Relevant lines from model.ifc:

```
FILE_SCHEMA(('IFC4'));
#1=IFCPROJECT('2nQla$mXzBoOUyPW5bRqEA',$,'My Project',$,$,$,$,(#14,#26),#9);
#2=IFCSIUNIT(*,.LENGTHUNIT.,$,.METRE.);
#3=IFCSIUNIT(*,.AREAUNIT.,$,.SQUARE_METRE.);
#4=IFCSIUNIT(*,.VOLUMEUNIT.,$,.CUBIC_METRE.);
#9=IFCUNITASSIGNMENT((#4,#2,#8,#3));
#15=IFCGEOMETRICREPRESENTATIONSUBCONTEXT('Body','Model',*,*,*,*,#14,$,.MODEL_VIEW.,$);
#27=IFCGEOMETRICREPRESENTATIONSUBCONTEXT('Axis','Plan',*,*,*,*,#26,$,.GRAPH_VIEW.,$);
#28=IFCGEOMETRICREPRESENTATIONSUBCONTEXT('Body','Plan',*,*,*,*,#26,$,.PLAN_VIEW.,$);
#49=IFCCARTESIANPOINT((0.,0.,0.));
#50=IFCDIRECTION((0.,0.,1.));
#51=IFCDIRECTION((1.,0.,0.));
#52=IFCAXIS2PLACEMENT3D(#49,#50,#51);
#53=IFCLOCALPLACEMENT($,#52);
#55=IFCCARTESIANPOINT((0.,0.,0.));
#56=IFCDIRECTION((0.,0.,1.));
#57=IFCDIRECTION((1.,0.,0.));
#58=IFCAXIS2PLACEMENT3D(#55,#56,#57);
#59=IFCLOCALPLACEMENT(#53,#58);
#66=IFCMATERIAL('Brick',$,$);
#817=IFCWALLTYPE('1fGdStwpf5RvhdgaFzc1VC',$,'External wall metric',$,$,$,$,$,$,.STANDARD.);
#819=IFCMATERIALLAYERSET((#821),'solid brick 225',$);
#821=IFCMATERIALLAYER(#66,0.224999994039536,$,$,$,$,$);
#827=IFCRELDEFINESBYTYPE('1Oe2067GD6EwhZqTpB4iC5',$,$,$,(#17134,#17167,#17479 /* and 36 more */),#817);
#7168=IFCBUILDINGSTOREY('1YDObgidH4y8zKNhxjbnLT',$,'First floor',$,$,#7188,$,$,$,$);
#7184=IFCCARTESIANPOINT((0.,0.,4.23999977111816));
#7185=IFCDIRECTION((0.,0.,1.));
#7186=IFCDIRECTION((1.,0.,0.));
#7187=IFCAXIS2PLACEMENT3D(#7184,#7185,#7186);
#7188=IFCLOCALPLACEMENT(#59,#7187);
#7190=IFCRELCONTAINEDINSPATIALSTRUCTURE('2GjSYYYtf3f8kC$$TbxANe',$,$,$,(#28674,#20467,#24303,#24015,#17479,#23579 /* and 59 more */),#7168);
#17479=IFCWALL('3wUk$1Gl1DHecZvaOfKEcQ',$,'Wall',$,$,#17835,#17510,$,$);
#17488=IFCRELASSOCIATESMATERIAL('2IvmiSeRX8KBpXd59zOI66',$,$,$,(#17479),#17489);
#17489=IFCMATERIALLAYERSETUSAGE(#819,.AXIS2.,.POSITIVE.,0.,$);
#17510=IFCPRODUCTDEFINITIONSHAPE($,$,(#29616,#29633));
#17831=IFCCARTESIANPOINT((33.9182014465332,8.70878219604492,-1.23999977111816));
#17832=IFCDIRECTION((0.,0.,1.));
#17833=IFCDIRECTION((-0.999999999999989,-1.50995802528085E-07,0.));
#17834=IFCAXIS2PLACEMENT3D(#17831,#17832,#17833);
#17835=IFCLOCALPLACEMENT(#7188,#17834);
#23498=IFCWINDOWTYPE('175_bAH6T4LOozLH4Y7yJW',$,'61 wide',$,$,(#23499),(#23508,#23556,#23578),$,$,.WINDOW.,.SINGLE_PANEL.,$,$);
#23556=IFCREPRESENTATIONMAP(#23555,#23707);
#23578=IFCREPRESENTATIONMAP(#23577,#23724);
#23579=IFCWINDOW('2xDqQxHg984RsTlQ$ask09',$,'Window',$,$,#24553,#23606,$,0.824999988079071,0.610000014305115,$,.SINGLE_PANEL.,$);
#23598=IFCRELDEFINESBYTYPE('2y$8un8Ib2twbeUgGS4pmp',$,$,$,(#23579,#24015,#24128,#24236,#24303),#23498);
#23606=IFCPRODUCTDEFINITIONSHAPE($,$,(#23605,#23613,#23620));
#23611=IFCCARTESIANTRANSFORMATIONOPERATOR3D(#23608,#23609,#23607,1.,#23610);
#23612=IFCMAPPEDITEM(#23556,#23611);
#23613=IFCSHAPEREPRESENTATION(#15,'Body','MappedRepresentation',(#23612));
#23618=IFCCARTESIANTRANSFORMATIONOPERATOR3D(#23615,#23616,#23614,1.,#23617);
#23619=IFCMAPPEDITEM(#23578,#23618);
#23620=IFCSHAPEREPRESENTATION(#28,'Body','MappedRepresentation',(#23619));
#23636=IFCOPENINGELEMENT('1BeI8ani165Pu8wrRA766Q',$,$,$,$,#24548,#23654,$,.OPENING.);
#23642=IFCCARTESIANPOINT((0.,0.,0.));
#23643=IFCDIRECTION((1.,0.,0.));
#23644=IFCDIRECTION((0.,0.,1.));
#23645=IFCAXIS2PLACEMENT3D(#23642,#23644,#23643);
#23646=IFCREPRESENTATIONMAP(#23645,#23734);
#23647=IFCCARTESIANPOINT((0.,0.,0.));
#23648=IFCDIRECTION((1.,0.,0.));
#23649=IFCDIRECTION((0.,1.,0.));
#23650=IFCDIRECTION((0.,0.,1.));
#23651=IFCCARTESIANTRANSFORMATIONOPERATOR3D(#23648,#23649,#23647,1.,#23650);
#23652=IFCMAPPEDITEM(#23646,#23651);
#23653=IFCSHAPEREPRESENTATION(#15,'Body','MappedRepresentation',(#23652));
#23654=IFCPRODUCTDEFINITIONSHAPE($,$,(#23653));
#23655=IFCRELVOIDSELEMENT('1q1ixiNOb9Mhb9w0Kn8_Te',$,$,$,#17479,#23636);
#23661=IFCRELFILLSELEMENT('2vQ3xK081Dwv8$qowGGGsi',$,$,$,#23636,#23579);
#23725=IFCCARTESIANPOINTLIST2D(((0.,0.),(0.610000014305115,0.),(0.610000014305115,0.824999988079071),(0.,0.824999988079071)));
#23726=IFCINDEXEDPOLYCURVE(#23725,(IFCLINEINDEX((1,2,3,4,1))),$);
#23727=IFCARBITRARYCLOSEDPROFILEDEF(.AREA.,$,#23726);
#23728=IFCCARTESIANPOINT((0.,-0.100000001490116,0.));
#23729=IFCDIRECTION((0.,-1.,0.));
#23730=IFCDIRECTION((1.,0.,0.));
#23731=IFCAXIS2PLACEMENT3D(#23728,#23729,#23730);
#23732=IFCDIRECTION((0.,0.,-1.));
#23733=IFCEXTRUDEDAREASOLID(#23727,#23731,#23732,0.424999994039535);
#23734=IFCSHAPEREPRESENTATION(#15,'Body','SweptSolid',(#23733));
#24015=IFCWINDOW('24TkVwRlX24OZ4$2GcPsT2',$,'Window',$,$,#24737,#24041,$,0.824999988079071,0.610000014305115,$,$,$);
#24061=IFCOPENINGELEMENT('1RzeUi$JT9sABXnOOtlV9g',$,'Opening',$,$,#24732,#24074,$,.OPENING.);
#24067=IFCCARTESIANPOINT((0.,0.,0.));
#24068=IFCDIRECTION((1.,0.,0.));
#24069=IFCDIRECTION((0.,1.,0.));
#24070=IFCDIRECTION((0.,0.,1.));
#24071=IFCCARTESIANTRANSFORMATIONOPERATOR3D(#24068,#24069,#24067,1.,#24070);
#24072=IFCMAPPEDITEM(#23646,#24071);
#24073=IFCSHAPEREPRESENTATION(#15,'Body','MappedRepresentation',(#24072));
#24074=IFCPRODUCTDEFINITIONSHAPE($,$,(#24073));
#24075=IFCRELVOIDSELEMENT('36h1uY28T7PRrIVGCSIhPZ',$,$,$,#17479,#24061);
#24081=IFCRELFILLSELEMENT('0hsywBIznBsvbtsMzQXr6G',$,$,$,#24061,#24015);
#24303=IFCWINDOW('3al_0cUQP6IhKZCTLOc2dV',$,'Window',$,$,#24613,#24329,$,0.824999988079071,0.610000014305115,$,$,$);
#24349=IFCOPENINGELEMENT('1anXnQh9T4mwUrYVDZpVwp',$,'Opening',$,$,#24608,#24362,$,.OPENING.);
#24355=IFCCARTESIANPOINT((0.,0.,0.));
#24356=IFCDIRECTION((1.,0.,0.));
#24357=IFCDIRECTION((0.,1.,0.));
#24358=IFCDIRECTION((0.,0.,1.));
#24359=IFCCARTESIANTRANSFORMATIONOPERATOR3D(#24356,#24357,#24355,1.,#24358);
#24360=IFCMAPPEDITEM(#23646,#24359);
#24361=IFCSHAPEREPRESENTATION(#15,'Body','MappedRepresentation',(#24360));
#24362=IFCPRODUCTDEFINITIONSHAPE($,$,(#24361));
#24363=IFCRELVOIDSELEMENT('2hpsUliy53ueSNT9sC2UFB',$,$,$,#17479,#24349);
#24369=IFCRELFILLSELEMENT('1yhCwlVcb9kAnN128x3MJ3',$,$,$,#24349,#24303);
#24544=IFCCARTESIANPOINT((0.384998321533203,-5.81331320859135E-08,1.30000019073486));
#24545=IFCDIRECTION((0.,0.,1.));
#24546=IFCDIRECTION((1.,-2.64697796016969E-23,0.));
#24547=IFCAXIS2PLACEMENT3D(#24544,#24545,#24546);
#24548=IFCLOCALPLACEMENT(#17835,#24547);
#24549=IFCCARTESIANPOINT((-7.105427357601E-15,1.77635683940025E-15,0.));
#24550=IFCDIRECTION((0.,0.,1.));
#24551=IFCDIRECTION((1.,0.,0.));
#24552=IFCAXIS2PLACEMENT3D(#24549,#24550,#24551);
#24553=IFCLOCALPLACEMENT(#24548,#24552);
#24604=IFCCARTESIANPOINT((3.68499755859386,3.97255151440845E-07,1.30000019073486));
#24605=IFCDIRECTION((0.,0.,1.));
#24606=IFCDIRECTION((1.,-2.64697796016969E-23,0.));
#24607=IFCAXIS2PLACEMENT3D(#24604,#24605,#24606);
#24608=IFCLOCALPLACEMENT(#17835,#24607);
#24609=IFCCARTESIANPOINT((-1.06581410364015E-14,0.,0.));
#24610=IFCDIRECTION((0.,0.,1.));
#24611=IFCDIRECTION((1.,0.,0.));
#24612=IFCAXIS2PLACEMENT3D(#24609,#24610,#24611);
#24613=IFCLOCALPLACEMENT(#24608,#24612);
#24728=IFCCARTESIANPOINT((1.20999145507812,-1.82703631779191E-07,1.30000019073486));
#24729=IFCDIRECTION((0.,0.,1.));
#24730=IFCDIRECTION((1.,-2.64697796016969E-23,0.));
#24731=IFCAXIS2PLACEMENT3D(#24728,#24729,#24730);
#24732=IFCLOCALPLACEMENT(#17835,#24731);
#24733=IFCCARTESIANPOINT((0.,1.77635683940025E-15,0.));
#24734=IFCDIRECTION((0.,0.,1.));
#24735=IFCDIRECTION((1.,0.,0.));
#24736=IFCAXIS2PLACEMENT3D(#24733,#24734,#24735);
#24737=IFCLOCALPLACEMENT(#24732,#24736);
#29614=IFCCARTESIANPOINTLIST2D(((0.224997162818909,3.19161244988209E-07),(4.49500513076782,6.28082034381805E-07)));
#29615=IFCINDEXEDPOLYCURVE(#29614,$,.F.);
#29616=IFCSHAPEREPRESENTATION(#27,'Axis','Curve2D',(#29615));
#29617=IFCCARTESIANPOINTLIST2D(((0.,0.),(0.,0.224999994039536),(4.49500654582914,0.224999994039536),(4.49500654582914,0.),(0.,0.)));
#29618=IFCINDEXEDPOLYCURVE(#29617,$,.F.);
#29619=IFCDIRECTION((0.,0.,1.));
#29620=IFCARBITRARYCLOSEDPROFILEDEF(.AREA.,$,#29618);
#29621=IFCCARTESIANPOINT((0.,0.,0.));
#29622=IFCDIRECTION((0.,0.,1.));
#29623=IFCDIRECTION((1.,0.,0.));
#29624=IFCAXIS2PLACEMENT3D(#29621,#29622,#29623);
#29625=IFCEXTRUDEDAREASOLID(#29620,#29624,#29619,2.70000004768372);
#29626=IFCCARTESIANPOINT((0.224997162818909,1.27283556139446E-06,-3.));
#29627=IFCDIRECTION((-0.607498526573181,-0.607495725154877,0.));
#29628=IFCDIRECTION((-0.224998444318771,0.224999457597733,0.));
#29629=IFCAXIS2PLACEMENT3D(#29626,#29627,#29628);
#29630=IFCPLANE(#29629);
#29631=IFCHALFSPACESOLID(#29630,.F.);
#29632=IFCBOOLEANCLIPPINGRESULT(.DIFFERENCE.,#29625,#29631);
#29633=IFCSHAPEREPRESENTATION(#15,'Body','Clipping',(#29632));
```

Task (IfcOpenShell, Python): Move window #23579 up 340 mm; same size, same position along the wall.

```python
import numpy as np
import ifcopenshell
import ifcopenshell.api.geometry
import ifcopenshell.util.placement
import ifcopenshell.util.unit

model = ifcopenshell.open("model.ifc")
unit_scale = ifcopenshell.util.unit.calculate_unit_scale(model)

window = model.by_id(23579)
opening = window.FillsVoids[0].RelatingOpeningElement
dz = 0.34

shift = np.array([0.0, 0.0, dz])
# The window is placed relative to its opening, so it follows when the opening moves.
matrix = ifcopenshell.util.placement.get_local_placement(opening.ObjectPlacement)
matrix[:3, 3] += shift
ifcopenshell.api.geometry.edit_object_placement(
    model, product=opening, matrix=matrix, is_si=False, should_transform_children=True
)

print(f"moved by {dz * unit_scale:+.3f} m")

model.write("model_v2.ifc")
```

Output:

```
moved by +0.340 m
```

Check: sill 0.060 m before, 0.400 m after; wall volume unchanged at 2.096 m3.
